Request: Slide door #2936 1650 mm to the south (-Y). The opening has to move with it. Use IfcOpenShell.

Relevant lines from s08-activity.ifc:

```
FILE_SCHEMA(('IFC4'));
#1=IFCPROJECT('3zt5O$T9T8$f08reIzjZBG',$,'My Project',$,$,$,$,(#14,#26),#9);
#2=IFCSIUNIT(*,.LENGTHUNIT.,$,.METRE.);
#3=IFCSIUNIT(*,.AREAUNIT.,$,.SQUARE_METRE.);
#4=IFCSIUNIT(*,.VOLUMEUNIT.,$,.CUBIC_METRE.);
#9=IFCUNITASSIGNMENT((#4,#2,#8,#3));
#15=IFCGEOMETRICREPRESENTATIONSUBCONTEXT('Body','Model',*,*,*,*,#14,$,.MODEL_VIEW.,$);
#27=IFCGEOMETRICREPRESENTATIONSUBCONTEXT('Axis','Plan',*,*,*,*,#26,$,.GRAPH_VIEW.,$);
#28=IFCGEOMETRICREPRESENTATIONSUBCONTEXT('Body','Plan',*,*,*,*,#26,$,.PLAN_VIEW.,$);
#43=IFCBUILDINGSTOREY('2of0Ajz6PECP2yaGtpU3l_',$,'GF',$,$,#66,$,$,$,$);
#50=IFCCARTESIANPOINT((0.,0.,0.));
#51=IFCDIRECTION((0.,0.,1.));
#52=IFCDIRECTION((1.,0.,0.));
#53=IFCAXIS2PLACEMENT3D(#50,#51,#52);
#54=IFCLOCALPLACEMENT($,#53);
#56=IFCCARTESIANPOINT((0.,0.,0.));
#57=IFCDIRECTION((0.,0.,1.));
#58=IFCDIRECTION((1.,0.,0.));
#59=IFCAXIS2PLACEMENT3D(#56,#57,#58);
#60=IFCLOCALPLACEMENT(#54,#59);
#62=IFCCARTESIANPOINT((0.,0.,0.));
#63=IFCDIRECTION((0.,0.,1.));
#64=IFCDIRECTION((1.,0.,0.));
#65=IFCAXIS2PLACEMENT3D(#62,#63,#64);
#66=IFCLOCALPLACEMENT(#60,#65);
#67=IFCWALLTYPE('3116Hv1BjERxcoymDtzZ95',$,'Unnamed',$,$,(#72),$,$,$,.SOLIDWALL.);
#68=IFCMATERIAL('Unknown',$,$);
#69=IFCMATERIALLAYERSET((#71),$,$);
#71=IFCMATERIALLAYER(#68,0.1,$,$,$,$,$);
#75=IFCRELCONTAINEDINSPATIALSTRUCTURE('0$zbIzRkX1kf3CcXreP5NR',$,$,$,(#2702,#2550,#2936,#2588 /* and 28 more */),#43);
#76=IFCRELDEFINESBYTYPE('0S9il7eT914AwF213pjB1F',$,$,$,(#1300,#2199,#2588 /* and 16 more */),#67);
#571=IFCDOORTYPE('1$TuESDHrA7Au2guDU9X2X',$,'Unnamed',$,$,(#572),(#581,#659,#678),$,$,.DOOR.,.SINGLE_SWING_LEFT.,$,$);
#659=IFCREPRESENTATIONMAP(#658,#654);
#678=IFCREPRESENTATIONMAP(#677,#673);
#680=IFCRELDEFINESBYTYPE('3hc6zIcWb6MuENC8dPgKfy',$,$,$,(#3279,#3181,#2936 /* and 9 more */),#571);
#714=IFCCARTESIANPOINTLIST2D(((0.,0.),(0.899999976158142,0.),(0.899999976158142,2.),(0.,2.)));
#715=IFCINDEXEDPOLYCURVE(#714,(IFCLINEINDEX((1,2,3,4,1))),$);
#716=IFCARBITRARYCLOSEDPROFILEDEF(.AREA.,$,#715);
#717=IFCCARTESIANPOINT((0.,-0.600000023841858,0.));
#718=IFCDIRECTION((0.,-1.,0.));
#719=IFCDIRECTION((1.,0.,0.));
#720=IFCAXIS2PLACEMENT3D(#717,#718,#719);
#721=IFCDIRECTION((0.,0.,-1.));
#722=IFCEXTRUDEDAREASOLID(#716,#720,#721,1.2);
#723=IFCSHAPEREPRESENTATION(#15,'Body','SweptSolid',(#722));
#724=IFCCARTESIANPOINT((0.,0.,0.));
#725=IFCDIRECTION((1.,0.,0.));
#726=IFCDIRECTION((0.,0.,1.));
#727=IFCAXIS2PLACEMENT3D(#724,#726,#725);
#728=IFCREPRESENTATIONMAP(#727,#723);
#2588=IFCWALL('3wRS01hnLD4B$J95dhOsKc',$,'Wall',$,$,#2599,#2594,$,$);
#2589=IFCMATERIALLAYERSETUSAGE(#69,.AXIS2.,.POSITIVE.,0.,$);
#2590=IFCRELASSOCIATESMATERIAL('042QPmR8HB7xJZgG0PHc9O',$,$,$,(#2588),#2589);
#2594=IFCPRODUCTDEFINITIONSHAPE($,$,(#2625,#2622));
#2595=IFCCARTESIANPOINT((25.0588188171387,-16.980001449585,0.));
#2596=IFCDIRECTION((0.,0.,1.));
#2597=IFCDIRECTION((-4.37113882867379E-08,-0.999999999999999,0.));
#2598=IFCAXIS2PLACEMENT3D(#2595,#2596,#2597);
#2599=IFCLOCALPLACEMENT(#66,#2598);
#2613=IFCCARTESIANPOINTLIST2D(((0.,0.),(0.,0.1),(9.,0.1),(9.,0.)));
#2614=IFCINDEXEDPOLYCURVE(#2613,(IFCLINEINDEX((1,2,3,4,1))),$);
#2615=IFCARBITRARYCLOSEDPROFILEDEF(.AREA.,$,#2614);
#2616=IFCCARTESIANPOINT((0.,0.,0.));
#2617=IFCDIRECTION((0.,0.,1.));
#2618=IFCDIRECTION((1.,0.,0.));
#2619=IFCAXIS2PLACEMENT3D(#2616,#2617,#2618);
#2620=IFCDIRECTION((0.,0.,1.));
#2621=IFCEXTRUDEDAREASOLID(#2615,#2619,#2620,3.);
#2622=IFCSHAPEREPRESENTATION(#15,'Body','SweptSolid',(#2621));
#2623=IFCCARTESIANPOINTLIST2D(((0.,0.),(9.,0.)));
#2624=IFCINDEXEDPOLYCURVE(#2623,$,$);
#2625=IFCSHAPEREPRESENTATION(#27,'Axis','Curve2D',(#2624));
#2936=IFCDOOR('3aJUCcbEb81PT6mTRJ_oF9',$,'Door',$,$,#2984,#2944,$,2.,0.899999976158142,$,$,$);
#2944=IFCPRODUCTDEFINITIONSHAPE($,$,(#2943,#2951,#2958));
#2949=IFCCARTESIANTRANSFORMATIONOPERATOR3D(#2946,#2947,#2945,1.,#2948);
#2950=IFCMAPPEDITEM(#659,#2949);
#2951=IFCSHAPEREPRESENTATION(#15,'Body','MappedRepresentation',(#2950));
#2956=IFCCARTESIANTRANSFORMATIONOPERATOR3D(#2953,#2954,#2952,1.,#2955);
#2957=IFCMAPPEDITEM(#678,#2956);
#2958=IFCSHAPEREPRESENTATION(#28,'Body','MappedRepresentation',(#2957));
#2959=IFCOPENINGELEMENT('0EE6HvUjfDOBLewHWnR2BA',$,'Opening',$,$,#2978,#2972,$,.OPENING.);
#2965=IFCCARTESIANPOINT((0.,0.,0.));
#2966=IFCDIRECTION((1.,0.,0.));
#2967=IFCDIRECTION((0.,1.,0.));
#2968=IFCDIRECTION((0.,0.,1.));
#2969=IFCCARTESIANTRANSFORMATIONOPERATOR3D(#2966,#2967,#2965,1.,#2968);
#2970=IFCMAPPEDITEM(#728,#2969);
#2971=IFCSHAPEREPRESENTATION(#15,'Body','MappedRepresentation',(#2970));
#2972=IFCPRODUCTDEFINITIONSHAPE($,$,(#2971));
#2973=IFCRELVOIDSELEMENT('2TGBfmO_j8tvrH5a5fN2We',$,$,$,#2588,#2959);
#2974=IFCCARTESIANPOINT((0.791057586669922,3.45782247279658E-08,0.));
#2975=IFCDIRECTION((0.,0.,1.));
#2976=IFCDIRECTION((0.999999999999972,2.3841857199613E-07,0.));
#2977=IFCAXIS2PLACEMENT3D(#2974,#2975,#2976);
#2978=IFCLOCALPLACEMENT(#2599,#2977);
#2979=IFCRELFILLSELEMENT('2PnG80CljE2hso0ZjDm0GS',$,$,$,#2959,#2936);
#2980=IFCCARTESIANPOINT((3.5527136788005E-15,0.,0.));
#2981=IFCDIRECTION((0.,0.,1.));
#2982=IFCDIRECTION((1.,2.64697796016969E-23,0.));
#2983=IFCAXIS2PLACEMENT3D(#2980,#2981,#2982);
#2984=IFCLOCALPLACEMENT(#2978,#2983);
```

```python
import ifcopenshell
import ifcopenshell.api.geometry
import ifcopenshell.util.placement

model = ifcopenshell.open("s08-activity.ifc")

door = model.by_guid("3aJUCcbEb81PT6mTRJ_oF9")
opening = door.FillsVoids[0].RelatingOpeningElement
wall = opening.VoidsElements[0].RelatingBuildingElement

wall_matrix = ifcopenshell.util.placement.get_local_placement(wall.ObjectPlacement)
shift = wall_matrix[:3, 0] * 1.65
before = ifcopenshell.util.placement.get_local_placement(door.ObjectPlacement)[:3, 3].copy()

# The door is placed relative to its opening, so it follows when the opening moves.
matrix = ifcopenshell.util.placement.get_local_placement(opening.ObjectPlacement)
matrix[:3, 3] += shift
ifcopenshell.api.geometry.edit_object_placement(
    model, product=opening, matrix=matrix, is_si=False, should_transform_children=True
)

after = ifcopenshell.util.placement.get_local_placement(door.ObjectPlacement)[:3, 3]
print("door moved by", (after - before).round(3) + 0.0)

model.write("s08-activity_edited.ifc")
```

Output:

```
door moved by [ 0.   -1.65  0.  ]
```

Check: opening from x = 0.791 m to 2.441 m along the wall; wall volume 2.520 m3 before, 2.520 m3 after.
